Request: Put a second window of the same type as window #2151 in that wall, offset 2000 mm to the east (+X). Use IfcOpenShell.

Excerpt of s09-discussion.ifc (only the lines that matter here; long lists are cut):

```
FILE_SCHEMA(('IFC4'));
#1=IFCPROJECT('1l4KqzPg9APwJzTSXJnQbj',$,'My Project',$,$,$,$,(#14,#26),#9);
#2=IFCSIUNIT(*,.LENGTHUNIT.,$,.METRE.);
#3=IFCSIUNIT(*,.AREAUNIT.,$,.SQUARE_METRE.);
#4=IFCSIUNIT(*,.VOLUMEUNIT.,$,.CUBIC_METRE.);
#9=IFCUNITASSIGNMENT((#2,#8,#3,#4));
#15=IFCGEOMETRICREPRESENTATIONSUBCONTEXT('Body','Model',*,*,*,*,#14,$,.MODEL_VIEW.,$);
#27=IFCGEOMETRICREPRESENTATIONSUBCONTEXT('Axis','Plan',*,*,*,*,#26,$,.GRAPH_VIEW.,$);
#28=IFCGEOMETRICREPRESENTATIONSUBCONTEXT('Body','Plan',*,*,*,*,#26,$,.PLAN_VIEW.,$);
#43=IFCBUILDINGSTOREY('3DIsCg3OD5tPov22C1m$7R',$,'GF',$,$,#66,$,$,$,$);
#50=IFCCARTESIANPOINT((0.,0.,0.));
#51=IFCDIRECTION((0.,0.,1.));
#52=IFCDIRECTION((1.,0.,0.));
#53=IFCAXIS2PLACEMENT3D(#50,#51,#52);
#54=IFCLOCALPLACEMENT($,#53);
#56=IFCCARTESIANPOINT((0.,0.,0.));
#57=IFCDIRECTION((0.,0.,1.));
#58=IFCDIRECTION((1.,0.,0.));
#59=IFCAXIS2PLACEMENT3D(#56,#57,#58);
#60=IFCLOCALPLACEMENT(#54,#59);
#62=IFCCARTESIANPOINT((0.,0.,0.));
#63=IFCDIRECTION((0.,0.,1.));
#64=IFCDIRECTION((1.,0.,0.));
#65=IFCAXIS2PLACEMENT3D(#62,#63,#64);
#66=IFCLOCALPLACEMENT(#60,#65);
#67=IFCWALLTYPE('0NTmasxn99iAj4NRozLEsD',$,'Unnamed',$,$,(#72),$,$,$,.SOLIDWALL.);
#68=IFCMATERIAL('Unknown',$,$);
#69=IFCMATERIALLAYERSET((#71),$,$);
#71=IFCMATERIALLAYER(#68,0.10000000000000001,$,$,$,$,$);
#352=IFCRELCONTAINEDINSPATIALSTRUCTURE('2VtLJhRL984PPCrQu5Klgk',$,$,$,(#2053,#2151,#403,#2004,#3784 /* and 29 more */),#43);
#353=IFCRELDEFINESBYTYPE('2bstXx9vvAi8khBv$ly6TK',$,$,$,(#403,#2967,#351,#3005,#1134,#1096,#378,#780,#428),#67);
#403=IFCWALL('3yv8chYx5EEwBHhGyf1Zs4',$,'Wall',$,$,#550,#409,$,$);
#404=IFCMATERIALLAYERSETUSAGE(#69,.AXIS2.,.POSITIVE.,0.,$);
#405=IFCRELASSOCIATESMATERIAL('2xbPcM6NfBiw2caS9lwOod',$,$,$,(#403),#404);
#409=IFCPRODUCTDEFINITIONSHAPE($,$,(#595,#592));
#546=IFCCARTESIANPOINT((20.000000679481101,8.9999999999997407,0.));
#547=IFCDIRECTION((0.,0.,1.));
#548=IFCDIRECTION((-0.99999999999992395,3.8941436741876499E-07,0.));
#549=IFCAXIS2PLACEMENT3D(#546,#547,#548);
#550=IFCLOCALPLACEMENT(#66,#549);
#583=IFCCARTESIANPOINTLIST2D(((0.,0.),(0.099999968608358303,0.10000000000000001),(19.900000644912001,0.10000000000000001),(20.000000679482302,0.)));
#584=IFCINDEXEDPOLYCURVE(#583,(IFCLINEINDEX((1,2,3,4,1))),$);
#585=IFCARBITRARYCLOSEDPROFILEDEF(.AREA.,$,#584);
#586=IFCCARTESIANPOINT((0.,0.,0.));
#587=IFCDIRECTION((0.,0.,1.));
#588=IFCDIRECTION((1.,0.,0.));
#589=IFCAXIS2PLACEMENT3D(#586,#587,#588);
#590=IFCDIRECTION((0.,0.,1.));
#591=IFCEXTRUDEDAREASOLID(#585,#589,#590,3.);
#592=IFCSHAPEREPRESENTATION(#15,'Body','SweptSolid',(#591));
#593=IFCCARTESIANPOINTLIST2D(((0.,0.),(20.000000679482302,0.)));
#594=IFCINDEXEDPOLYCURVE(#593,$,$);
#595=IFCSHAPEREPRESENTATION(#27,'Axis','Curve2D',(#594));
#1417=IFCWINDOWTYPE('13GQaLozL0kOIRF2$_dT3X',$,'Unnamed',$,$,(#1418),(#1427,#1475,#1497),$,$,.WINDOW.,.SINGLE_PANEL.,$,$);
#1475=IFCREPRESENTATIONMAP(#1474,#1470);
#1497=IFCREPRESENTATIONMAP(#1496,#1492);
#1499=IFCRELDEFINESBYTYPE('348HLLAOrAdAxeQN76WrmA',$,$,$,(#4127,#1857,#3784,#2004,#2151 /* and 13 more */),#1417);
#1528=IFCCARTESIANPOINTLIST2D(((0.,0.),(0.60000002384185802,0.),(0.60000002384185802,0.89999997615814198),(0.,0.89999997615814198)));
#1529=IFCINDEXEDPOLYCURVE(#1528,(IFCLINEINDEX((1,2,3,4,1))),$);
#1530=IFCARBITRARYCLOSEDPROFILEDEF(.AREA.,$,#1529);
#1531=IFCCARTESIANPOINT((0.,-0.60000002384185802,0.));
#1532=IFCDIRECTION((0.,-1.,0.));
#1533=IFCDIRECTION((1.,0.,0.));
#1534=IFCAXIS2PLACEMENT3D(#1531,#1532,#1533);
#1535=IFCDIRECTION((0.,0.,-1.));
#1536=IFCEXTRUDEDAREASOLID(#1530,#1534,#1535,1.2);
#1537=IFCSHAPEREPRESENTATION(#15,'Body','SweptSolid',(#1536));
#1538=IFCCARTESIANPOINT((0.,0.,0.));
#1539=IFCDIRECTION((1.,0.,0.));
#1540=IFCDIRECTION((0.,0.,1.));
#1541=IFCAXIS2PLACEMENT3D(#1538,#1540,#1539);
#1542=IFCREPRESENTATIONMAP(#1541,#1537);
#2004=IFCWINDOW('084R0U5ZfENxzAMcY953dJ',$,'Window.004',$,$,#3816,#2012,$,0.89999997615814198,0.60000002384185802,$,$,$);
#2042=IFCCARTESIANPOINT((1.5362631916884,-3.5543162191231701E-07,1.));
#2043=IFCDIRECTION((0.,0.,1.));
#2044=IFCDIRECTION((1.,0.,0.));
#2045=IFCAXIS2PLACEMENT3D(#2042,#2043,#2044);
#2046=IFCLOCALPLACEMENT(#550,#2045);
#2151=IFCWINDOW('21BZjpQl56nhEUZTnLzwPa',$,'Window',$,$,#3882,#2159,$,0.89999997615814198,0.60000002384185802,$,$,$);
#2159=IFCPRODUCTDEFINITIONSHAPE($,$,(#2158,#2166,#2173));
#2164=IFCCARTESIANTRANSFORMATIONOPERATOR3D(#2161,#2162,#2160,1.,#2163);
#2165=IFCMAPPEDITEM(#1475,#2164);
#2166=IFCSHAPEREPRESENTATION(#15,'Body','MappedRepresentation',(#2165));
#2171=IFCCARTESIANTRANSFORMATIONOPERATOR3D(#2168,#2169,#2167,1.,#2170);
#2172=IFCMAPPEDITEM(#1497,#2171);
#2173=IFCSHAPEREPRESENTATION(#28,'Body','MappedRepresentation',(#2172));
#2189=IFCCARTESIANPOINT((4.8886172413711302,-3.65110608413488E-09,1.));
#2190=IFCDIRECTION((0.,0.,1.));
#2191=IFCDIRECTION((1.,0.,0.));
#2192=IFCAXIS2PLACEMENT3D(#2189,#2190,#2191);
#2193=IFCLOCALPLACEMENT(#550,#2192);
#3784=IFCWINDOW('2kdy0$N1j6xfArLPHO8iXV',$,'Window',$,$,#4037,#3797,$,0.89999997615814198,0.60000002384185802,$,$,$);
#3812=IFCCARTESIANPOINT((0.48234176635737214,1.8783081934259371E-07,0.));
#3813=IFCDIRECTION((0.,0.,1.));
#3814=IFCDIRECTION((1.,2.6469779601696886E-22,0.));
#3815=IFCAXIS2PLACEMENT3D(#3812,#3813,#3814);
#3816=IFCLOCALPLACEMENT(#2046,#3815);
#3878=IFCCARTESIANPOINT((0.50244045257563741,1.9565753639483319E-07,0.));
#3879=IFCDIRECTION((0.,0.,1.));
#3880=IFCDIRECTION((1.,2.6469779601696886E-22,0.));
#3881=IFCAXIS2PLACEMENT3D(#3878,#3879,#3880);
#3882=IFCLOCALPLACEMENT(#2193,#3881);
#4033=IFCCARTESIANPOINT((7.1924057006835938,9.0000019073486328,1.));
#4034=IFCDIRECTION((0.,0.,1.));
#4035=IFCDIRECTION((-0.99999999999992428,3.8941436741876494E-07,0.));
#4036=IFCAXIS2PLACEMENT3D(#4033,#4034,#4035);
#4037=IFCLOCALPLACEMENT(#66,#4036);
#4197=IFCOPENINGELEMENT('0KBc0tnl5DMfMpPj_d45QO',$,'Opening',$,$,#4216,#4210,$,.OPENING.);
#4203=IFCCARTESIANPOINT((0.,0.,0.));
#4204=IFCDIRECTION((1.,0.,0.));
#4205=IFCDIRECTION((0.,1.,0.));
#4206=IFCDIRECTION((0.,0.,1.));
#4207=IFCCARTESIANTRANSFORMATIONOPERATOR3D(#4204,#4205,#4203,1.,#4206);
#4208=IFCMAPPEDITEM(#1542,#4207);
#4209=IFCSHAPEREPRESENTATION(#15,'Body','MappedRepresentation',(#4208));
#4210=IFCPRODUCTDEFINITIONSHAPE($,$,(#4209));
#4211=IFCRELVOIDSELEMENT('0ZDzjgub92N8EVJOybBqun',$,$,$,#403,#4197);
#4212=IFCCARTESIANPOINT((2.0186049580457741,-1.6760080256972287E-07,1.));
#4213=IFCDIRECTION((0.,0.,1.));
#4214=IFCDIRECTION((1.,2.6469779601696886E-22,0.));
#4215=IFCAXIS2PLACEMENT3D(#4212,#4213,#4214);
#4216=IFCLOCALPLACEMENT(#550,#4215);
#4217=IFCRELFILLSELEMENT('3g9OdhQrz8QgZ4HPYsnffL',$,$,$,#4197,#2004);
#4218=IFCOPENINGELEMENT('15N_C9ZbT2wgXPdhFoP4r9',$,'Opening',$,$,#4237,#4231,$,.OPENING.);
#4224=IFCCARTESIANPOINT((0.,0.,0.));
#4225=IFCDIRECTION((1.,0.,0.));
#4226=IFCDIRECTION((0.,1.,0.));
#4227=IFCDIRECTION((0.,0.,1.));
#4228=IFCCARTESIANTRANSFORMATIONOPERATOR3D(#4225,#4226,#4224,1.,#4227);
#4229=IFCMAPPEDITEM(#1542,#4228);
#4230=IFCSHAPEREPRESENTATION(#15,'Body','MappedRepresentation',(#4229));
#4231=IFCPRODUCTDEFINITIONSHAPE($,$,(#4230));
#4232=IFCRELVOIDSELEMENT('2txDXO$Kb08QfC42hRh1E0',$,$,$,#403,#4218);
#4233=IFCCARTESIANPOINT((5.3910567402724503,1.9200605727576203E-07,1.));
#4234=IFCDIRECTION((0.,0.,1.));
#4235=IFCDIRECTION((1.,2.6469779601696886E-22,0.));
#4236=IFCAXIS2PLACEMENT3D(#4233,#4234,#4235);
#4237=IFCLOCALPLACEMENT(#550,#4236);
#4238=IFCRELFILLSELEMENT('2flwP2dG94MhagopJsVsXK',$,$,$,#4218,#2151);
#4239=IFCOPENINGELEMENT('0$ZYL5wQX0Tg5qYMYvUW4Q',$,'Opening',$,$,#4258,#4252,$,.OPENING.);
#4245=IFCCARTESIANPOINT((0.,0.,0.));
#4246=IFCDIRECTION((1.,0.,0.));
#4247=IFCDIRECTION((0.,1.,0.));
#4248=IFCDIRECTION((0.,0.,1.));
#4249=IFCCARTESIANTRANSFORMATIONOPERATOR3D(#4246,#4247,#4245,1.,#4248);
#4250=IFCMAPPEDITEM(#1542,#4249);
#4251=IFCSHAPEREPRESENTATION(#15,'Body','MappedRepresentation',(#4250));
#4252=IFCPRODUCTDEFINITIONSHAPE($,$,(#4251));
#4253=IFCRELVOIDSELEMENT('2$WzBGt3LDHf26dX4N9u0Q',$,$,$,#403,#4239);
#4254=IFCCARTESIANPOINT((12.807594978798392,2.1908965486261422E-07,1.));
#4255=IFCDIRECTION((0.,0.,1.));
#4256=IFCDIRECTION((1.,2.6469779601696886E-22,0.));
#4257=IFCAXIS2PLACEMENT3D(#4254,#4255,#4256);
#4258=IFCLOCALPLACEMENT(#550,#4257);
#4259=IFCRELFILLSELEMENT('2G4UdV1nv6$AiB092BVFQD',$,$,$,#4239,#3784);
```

```python
import ifcopenshell
import ifcopenshell.api.feature
import ifcopenshell.api.geometry
import ifcopenshell.api.root
import ifcopenshell.geom
import ifcopenshell.util.element
import ifcopenshell.util.placement
import ifcopenshell.util.shape
import ifcopenshell.util.unit

model = ifcopenshell.open("s09-discussion.ifc")
unit_scale = ifcopenshell.util.unit.calculate_unit_scale(model)
settings = ifcopenshell.geom.settings()


def volume(element):
    """Net volume in cubic metres, openings subtracted."""
    shape = ifcopenshell.geom.create_shape(settings, element)
    return ifcopenshell.util.shape.get_volume(shape.geometry)


window = model.by_id(2151)
opening = window.FillsVoids[0].RelatingOpeningElement
wall = opening.VoidsElements[0].RelatingBuildingElement
before = volume(wall)
shift = ifcopenshell.util.placement.get_local_placement(wall.ObjectPlacement)[:3, 0] * -2 / unit_scale

# copy_class copies the void relationship, type, container and properties, but no geometry.
new_opening = ifcopenshell.api.root.copy_class(model, product=opening)
new_opening.Representation = ifcopenshell.util.element.copy_deep(
    model, opening.Representation, exclude=["IfcGeometricRepresentationContext", "IfcRepresentationMap"]
)
new_window = ifcopenshell.api.root.copy_class(model, product=window)
new_window.Representation = ifcopenshell.util.element.copy_deep(
    model, window.Representation, exclude=["IfcGeometricRepresentationContext", "IfcRepresentationMap"]
)
ifcopenshell.api.feature.add_filling(model, opening=new_opening, element=new_window)

for old, new in ((opening, new_opening), (window, new_window)):
    matrix = ifcopenshell.util.placement.get_local_placement(old.ObjectPlacement)
    matrix[:3, 3] += shift
    ifcopenshell.api.geometry.edit_object_placement(model, product=new, matrix=matrix, is_si=False)

after = volume(wall)

print(f"wall volume {before:.3f} -> {after:.3f} m3")

model.write("s09-discussion_edited.ifc")
```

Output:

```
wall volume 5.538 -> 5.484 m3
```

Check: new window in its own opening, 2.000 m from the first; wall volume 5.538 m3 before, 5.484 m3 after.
